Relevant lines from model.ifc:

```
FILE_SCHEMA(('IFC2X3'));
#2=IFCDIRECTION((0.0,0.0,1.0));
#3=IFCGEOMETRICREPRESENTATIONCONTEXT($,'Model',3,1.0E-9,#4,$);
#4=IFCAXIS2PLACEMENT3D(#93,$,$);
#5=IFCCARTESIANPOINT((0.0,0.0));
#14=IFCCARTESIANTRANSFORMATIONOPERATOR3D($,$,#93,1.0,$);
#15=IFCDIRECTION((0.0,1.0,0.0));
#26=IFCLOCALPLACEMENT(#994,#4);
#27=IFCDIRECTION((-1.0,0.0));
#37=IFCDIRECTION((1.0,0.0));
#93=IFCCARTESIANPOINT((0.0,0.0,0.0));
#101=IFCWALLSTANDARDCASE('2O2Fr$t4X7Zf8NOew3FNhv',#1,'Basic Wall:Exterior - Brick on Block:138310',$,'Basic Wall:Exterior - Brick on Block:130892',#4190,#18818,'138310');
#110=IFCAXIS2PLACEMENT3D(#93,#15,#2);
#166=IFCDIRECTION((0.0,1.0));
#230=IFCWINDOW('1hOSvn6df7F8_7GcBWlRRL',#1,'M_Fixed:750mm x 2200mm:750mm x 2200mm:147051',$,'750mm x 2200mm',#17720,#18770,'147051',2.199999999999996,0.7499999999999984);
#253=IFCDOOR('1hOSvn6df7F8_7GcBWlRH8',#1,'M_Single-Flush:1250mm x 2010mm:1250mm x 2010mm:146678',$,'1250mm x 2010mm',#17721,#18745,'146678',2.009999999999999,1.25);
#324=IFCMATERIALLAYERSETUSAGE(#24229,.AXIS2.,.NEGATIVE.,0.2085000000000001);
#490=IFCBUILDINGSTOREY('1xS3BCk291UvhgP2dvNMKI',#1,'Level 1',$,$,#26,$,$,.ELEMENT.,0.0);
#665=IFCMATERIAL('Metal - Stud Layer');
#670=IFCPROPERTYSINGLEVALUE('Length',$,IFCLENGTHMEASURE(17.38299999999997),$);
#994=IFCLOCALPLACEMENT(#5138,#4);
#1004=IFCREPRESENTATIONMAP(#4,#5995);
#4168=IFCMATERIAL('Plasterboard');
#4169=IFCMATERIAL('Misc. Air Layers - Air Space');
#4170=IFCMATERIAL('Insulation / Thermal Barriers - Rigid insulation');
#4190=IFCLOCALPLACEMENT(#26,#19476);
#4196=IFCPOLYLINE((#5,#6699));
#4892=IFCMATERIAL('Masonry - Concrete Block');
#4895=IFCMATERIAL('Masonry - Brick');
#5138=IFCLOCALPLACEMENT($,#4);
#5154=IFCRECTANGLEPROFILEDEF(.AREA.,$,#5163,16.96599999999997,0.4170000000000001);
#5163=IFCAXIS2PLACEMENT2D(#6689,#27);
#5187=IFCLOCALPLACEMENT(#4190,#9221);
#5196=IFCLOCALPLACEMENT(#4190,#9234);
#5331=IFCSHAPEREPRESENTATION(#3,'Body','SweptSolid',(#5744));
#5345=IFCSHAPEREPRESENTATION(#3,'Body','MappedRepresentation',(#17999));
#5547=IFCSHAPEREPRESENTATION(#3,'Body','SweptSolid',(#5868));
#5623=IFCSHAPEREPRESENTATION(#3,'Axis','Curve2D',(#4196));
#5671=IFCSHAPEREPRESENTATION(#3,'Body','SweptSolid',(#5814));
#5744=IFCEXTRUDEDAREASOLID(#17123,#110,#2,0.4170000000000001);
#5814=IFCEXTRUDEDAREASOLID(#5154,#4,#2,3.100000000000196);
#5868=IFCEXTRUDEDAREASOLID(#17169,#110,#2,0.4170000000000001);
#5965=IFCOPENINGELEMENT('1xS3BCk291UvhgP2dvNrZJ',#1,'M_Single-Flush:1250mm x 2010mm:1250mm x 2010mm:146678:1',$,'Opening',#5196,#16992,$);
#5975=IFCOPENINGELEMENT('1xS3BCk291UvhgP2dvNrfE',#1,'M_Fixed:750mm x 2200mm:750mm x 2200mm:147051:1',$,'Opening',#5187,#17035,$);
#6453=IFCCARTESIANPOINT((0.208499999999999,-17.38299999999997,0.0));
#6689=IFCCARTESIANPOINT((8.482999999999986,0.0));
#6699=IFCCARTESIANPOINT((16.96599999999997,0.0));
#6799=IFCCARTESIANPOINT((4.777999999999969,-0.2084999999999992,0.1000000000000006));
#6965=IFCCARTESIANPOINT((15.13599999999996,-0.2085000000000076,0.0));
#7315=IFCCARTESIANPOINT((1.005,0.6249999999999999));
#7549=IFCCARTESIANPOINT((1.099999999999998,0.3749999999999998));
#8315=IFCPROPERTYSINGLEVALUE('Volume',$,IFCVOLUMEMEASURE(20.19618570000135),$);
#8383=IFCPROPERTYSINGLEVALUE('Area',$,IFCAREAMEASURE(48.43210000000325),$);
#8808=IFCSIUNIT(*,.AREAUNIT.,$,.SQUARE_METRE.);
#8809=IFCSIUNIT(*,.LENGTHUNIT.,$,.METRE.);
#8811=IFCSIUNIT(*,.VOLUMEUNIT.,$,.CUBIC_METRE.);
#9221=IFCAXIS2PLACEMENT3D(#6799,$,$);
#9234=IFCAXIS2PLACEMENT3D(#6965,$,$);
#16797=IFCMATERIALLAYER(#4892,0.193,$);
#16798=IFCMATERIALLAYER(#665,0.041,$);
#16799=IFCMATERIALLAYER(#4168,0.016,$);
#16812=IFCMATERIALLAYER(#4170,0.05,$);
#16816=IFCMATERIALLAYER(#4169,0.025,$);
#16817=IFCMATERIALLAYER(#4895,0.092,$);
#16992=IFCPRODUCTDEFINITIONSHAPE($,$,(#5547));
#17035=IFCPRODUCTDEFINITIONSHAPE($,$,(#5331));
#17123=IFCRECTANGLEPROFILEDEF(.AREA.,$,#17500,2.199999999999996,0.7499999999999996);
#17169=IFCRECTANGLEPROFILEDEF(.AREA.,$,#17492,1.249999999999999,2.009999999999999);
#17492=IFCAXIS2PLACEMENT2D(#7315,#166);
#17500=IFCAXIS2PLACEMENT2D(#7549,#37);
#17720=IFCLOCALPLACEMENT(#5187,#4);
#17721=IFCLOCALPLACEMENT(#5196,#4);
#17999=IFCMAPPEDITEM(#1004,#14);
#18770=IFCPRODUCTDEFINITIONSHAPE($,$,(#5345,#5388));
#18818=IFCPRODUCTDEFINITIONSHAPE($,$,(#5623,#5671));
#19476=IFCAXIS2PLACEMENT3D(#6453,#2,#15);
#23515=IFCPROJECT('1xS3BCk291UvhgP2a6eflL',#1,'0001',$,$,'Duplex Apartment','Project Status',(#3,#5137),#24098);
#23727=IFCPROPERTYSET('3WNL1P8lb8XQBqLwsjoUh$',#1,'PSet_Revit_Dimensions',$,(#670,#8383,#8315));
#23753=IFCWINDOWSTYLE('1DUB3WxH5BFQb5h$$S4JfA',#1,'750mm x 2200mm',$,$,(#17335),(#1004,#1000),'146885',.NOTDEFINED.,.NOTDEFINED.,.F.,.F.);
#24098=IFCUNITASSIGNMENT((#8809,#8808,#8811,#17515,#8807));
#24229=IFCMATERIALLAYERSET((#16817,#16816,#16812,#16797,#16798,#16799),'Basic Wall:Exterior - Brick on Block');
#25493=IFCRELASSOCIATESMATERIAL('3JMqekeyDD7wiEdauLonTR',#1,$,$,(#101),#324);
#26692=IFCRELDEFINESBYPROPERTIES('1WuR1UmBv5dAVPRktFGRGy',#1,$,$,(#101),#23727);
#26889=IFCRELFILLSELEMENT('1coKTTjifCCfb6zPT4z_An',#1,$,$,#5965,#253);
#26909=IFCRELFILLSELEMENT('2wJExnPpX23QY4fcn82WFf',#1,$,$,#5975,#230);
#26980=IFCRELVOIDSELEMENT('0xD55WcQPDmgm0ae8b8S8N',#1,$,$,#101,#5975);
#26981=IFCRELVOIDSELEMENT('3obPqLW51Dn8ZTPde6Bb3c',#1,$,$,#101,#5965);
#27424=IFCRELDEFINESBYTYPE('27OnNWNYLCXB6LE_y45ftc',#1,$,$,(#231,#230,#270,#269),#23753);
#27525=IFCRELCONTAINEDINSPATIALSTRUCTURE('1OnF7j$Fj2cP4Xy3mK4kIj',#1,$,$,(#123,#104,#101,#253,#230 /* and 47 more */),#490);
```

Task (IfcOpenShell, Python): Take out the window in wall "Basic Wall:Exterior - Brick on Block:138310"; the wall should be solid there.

```python
import ifcopenshell
import ifcopenshell.api.feature
import ifcopenshell.api.pset
import ifcopenshell.api.root
import ifcopenshell.geom
import ifcopenshell.util.element
import ifcopenshell.util.shape
import ifcopenshell.util.unit

model = ifcopenshell.open("model.ifc")
area_scale = ifcopenshell.util.unit.calculate_unit_scale(model, "AREAUNIT")
volume_scale = ifcopenshell.util.unit.calculate_unit_scale(model, "VOLUMEUNIT")
settings = ifcopenshell.geom.settings()


def volume(element):
    """Net volume in cubic metres, openings subtracted."""
    shape = ifcopenshell.geom.create_shape(settings, element)
    return ifcopenshell.util.shape.get_volume(shape.geometry)


window = model.by_guid("1hOSvn6df7F8_7GcBWlRRL")
opening = window.FillsVoids[0].RelatingOpeningElement
wall = opening.VoidsElements[0].RelatingBuildingElement
before = volume(wall)

ifcopenshell.api.root.remove_product(model, product=window)
ifcopenshell.api.feature.remove_feature(model, feature=opening)

after = volume(wall)
thickness = 0.417  # wall thickness in metres

# Update the wall's stored quantities.
pset = model.by_id(ifcopenshell.util.element.get_pset(wall, "PSet_Revit_Dimensions", should_inherit=False)["id"])
ifcopenshell.api.pset.edit_pset(model, pset=pset, properties={
    "Area": model.create_entity("IfcAreaMeasure", after / thickness / area_scale),
    "Volume": model.create_entity("IfcVolumeMeasure", after / volume_scale),
})

print(f"wall volume {before:.3f} -> {after:.3f} m3")

model.write("model-out.ifc")
```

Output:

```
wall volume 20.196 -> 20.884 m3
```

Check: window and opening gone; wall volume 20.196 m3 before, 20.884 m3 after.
